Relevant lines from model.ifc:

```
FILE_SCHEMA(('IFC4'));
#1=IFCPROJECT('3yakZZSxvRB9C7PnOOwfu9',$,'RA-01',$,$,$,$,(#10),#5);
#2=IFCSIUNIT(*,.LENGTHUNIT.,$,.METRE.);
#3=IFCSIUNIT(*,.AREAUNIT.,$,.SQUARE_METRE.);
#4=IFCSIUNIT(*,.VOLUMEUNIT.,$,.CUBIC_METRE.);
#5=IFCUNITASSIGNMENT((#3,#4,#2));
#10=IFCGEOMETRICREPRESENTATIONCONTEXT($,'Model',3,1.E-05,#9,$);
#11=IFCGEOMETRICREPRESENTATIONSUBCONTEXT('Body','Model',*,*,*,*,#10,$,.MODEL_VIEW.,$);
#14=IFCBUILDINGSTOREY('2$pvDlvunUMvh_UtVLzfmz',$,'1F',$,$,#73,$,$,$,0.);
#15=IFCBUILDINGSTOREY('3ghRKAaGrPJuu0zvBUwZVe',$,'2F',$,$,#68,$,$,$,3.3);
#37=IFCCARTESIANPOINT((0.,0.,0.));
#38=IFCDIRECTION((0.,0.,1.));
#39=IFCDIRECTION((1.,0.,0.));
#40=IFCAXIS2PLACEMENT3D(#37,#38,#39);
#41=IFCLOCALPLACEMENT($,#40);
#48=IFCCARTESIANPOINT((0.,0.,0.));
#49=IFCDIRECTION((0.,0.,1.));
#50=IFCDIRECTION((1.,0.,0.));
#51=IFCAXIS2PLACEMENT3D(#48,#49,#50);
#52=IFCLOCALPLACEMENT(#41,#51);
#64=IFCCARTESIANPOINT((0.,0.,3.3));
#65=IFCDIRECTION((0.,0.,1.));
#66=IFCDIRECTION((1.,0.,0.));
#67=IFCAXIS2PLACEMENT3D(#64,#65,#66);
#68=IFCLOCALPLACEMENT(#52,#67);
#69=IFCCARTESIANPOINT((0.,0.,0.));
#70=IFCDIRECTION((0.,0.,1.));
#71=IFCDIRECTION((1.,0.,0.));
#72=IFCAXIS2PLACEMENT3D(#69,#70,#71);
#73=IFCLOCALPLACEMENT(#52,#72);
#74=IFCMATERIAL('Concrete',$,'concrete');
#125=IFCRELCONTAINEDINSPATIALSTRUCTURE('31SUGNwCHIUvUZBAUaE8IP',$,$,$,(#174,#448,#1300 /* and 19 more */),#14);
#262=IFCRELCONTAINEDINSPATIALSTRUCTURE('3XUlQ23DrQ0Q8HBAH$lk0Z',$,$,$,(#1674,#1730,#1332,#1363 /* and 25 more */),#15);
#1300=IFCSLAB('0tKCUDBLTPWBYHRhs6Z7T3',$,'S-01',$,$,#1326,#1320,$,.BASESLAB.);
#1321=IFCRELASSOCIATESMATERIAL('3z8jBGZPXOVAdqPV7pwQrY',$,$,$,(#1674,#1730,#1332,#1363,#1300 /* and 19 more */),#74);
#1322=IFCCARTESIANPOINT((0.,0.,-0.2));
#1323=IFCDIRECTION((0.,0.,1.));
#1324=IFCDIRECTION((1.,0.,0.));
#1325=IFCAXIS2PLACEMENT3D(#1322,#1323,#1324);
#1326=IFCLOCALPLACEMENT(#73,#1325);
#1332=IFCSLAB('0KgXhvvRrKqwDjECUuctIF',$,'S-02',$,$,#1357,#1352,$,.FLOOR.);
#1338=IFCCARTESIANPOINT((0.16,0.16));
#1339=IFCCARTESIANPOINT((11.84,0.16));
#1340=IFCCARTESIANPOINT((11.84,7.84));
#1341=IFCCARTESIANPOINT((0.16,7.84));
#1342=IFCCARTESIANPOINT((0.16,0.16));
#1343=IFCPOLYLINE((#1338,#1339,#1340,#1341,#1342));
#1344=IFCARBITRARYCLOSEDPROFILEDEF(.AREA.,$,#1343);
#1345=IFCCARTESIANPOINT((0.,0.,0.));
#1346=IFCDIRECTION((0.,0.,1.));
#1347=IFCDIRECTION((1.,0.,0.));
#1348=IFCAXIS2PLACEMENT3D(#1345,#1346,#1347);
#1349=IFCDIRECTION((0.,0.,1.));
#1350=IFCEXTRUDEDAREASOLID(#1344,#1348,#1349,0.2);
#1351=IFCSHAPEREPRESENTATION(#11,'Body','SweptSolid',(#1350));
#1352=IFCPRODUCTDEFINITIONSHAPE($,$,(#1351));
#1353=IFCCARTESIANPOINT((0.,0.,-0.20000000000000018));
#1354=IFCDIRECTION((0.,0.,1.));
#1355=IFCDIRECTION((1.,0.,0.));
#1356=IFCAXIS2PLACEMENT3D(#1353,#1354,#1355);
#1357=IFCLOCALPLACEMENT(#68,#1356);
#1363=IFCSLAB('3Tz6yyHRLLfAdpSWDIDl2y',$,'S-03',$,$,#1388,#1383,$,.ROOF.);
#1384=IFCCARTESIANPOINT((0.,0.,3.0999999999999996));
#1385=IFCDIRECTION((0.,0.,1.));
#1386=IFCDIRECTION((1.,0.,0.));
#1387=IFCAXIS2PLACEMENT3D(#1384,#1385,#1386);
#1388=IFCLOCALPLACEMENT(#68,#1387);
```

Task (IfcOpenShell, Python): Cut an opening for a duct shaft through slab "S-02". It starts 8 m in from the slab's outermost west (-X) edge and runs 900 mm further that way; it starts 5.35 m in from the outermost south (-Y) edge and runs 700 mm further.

```python
import numpy as np
import ifcopenshell
import ifcopenshell.api.feature
import ifcopenshell.api.geometry
import ifcopenshell.api.root
import ifcopenshell.geom
import ifcopenshell.util.placement
import ifcopenshell.util.representation
import ifcopenshell.util.shape
import ifcopenshell.util.unit

model = ifcopenshell.open("model.ifc")
unit_scale = ifcopenshell.util.unit.calculate_unit_scale(model)
settings = ifcopenshell.geom.settings()


def volume(element):
    """Net volume in cubic metres, openings subtracted."""
    shape = ifcopenshell.geom.create_shape(settings, element)
    return ifcopenshell.util.shape.get_volume(shape.geometry)


slab = model.by_guid("0KgXhvvRrKqwDjECUuctIF")
before = volume(slab)

# Extent in the slab's own axes, in metres. The edges named are its -X and -Y sides.
slab_shape = ifcopenshell.geom.create_shape(settings, slab)
vertices = ifcopenshell.util.shape.get_vertices(slab_shape.geometry)
x_min, y_min, bottom = vertices.min(axis=0)
top = vertices[:, 2].max()

opening = ifcopenshell.api.root.create_entity(model, ifc_class="IfcOpeningElement", name="Duct shaft opening", predefined_type="OPENING")
context = ifcopenshell.util.representation.get_context(model, "Model", "Body", "MODEL_VIEW")
width, depth = 0.9, 0.7
outline = [(0.0, 0.0), (width, 0.0), (width, depth), (0.0, depth), (0.0, 0.0)]
# Overshoot both faces by 50 mm so the cut is clean.
shape = ifcopenshell.api.geometry.add_slab_representation(
    model, context=context, depth=top - bottom + 0.1, polyline=outline
)
ifcopenshell.api.geometry.assign_representation(model, product=opening, representation=shape)

matrix = ifcopenshell.util.placement.get_local_placement(slab.ObjectPlacement)
matrix[:, 3] = matrix @ np.append(np.array([x_min + 8, y_min + 5.35, bottom - 0.05]) / unit_scale, 1.0)
ifcopenshell.api.geometry.edit_object_placement(model, product=opening, matrix=matrix, is_si=False)
ifcopenshell.api.feature.add_feature(model, feature=opening, element=slab)

after = volume(slab)

print(f"slab volume {before:.3f} -> {after:.3f} m3")

model.write("model_edited.ifc")
```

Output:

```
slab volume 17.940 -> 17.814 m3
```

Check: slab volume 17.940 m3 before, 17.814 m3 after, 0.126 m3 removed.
